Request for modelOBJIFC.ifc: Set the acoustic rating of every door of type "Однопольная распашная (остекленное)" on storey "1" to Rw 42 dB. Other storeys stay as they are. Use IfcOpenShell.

First a look at what the model holds.

```python
import ifcopenshell
import ifcopenshell.util.element

model = ifcopenshell.open("modelOBJIFC.ifc")
print(model.schema)
storey = next(s for s in model.by_type("IfcBuildingStorey") if s.Name == "1")
doors = [e for e in ifcopenshell.util.element.get_decomposition(storey) if e.is_a("IfcDoor")]
seen = {}
for e in doors:
    element_type = ifcopenshell.util.element.get_type(e)
    key = (element_type.Name if element_type != e and element_type else None, ifcopenshell.util.element.get_pset(e, "Pset_DoorCommon", "AcousticRating"))
    seen[key] = seen.get(key, 0) + 1
for (name, value), count in sorted(seen.items(), key=str):
    print(count, "x", name, "|", value)
```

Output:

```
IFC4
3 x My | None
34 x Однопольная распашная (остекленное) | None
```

```python
import ifcopenshell
import ifcopenshell.api.pset
import ifcopenshell.util.element

model = ifcopenshell.open("modelOBJIFC.ifc")

storey = next(s for s in model.by_type("IfcBuildingStorey") if s.Name == "1")
doors = [e for e in ifcopenshell.util.element.get_decomposition(storey) if e.is_a("IfcDoor")]

count = 0
for e in doors:
    element_type = ifcopenshell.util.element.get_type(e)
    if element_type in (None, e) or element_type.Name != "Однопольная распашная (остекленное)":
        continue
    # add_pset returns the element's existing set when there is one.
    pset = ifcopenshell.api.pset.add_pset(model, product=e, name="Pset_DoorCommon")
    ifcopenshell.api.pset.edit_pset(model, pset=pset, properties={"AcousticRating": "Rw 42 dB"})
    count += 1

print(count, "doors updated")

model.write("modelOBJIFC_edited.ifc")
```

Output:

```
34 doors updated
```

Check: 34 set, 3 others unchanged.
